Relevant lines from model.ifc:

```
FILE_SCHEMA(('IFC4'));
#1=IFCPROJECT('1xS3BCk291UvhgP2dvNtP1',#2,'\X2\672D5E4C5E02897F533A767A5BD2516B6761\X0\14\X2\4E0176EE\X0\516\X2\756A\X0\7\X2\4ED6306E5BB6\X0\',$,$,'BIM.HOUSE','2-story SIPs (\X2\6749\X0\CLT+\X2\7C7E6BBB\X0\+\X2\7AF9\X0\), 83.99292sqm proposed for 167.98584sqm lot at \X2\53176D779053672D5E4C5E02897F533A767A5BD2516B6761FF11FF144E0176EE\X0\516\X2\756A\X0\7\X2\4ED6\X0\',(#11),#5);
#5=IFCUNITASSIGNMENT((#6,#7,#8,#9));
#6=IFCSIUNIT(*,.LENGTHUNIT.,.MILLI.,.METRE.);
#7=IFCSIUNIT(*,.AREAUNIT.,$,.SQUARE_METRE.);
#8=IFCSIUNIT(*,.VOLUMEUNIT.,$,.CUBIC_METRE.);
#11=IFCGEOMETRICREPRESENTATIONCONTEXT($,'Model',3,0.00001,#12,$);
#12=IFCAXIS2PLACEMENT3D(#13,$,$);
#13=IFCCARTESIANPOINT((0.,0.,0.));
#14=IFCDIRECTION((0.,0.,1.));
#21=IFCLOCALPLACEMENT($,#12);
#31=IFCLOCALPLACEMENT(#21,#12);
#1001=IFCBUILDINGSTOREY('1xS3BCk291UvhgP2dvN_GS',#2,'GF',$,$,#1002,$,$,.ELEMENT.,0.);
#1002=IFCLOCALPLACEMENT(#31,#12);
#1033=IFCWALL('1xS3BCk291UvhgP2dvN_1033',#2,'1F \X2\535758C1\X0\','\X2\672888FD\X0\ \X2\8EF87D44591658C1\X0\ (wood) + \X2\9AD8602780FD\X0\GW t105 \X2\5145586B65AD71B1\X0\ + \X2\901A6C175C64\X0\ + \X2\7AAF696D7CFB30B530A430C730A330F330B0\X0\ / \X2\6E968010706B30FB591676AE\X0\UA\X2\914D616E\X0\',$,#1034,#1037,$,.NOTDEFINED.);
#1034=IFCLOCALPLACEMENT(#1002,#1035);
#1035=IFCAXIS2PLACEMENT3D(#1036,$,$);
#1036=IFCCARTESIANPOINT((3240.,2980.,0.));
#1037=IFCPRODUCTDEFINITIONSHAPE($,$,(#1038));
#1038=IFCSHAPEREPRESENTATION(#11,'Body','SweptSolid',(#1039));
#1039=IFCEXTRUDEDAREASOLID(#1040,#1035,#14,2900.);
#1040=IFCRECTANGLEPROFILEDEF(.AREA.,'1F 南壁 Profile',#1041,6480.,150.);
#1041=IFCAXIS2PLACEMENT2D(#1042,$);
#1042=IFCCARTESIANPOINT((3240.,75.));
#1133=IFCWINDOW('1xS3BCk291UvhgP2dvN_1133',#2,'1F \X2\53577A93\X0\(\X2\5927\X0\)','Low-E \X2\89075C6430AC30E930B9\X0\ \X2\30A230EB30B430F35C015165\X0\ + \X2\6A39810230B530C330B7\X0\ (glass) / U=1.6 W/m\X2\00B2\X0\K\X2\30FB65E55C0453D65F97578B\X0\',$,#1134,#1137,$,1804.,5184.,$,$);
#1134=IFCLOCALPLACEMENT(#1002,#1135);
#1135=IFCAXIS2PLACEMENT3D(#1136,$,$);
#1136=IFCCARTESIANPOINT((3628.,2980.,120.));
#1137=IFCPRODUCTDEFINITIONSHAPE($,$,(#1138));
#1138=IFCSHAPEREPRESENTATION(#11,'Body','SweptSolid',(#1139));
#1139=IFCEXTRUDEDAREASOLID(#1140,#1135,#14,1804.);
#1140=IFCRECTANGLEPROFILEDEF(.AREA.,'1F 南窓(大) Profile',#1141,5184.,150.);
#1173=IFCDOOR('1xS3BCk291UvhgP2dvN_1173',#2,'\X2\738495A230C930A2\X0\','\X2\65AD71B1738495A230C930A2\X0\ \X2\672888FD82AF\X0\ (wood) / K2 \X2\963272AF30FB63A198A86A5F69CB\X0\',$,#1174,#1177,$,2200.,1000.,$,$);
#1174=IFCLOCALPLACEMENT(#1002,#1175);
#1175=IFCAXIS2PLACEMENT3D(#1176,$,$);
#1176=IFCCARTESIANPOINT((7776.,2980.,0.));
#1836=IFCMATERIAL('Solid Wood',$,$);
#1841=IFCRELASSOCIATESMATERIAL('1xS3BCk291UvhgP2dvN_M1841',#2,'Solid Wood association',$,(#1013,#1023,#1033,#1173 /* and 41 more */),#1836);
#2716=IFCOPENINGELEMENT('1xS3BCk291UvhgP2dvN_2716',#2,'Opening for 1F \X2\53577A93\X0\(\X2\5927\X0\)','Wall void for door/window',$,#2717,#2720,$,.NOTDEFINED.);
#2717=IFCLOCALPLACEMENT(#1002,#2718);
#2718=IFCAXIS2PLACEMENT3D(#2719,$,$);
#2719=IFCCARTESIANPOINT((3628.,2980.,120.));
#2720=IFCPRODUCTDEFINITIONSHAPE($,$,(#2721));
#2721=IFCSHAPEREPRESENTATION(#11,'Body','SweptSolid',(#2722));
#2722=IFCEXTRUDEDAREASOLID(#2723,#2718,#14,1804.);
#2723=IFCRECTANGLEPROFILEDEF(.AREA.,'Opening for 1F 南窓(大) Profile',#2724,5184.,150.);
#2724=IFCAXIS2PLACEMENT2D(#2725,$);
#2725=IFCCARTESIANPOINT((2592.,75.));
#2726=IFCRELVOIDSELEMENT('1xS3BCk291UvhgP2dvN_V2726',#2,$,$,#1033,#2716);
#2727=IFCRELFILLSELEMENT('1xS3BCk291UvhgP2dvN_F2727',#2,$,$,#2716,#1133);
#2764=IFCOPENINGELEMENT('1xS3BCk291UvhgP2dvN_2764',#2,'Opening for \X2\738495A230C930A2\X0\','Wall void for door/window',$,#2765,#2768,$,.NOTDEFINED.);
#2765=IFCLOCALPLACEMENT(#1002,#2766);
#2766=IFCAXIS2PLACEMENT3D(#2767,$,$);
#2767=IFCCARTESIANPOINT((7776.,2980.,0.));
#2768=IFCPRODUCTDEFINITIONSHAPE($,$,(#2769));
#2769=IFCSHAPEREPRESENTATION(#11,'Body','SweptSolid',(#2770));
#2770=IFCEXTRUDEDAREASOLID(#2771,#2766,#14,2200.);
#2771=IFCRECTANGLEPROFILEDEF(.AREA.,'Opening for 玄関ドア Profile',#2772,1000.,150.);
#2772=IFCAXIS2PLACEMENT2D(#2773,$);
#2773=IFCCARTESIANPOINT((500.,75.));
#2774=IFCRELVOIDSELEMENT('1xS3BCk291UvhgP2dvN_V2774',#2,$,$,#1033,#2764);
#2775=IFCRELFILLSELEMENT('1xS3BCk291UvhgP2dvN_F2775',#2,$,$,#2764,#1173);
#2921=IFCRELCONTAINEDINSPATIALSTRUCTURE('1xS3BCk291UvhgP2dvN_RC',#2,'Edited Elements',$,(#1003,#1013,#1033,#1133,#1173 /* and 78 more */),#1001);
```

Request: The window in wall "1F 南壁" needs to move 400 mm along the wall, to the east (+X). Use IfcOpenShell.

```python
import ifcopenshell
import ifcopenshell.api.geometry
import ifcopenshell.util.placement
import ifcopenshell.util.unit

model = ifcopenshell.open("model.ifc")
unit_scale = ifcopenshell.util.unit.calculate_unit_scale(model)

window = model.by_guid("1xS3BCk291UvhgP2dvN_1133")
opening = window.FillsVoids[0].RelatingOpeningElement
wall = opening.VoidsElements[0].RelatingBuildingElement

wall_matrix = ifcopenshell.util.placement.get_local_placement(wall.ObjectPlacement)
shift = wall_matrix[:3, 0] * 0.4 / unit_scale
before = ifcopenshell.util.placement.get_local_placement(window.ObjectPlacement)[:3, 3].copy()

# The window is not placed relative to its opening, so move both.
for product in (opening, window):
    matrix = ifcopenshell.util.placement.get_local_placement(product.ObjectPlacement)
    matrix[:3, 3] += shift
    ifcopenshell.api.geometry.edit_object_placement(model, product=product, matrix=matrix, is_si=False)

after = ifcopenshell.util.placement.get_local_placement(window.ObjectPlacement)[:3, 3]
print("window moved by", (after - before).round(3) + 0.0)

model.write("model_rev.ifc")
```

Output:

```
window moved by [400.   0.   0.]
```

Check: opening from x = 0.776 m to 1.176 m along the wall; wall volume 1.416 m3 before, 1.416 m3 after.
